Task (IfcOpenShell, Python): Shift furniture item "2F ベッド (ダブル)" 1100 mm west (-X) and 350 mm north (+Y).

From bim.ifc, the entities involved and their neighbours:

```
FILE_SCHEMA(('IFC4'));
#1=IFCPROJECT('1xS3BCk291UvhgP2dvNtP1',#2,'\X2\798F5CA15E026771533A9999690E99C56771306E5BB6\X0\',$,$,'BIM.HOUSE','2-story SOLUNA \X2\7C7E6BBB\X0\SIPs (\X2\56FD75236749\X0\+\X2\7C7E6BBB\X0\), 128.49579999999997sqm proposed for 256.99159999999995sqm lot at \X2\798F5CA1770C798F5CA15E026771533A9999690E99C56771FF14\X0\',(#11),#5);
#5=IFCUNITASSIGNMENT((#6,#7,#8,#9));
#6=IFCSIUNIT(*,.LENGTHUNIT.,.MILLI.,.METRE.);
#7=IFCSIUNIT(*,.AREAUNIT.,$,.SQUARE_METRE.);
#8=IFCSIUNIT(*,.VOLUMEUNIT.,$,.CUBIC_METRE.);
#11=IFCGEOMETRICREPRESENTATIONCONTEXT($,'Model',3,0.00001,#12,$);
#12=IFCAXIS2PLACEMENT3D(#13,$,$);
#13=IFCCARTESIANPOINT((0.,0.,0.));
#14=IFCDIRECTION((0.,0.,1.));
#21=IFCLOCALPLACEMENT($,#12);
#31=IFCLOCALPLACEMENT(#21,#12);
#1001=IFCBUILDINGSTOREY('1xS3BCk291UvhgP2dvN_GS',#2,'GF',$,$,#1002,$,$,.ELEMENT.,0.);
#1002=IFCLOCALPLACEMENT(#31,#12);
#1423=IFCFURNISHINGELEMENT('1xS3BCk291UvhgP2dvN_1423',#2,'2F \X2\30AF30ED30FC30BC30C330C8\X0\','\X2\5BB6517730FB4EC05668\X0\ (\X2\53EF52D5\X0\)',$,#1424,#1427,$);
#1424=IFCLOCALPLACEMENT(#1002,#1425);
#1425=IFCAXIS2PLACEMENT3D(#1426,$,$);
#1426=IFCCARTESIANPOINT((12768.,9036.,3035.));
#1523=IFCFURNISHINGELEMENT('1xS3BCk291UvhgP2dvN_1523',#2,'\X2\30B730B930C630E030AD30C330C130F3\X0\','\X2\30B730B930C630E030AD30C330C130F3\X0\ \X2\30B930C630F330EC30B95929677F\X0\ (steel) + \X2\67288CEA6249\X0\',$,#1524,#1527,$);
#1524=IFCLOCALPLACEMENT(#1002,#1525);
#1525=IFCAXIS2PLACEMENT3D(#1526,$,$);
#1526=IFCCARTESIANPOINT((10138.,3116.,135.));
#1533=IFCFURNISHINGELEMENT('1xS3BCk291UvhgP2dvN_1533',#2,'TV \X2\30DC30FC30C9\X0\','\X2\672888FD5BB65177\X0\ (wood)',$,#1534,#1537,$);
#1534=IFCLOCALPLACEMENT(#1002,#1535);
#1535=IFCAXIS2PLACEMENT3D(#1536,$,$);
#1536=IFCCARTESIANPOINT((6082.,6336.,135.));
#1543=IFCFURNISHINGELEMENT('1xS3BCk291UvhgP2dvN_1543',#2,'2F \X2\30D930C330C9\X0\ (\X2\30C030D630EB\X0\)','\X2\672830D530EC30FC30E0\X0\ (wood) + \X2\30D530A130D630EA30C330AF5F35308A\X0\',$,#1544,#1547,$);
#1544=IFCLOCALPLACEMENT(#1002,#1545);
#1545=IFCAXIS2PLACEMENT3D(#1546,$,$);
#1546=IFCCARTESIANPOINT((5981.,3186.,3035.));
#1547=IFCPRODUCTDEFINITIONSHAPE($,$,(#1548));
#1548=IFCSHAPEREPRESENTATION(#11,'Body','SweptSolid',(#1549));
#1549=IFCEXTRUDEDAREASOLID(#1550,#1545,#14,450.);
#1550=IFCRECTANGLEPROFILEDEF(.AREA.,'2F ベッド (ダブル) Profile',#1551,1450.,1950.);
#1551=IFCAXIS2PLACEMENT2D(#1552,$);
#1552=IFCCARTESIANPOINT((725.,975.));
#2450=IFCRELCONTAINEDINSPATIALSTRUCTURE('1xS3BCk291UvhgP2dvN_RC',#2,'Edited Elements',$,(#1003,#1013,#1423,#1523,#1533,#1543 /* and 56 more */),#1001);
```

```python
import ifcopenshell
import ifcopenshell.api.geometry
import ifcopenshell.util.placement
import ifcopenshell.util.unit

model = ifcopenshell.open("bim.ifc")
unit_scale = ifcopenshell.util.unit.calculate_unit_scale(model)

item = model.by_guid("1xS3BCk291UvhgP2dvN_1543")
matrix = ifcopenshell.util.placement.get_local_placement(item.ObjectPlacement)
matrix[0, 3] -= 1.1 / unit_scale
matrix[1, 3] += 0.35 / unit_scale
ifcopenshell.api.geometry.edit_object_placement(model, product=item, matrix=matrix, is_si=False)

print(ifcopenshell.util.placement.get_local_placement(item.ObjectPlacement).round(3) + 0.0)

model.write("bim_edited.ifc")
```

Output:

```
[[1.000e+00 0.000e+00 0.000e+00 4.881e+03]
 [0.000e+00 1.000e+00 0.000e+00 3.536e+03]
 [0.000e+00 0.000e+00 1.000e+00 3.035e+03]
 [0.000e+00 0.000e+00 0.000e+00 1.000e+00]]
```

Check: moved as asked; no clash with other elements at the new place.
